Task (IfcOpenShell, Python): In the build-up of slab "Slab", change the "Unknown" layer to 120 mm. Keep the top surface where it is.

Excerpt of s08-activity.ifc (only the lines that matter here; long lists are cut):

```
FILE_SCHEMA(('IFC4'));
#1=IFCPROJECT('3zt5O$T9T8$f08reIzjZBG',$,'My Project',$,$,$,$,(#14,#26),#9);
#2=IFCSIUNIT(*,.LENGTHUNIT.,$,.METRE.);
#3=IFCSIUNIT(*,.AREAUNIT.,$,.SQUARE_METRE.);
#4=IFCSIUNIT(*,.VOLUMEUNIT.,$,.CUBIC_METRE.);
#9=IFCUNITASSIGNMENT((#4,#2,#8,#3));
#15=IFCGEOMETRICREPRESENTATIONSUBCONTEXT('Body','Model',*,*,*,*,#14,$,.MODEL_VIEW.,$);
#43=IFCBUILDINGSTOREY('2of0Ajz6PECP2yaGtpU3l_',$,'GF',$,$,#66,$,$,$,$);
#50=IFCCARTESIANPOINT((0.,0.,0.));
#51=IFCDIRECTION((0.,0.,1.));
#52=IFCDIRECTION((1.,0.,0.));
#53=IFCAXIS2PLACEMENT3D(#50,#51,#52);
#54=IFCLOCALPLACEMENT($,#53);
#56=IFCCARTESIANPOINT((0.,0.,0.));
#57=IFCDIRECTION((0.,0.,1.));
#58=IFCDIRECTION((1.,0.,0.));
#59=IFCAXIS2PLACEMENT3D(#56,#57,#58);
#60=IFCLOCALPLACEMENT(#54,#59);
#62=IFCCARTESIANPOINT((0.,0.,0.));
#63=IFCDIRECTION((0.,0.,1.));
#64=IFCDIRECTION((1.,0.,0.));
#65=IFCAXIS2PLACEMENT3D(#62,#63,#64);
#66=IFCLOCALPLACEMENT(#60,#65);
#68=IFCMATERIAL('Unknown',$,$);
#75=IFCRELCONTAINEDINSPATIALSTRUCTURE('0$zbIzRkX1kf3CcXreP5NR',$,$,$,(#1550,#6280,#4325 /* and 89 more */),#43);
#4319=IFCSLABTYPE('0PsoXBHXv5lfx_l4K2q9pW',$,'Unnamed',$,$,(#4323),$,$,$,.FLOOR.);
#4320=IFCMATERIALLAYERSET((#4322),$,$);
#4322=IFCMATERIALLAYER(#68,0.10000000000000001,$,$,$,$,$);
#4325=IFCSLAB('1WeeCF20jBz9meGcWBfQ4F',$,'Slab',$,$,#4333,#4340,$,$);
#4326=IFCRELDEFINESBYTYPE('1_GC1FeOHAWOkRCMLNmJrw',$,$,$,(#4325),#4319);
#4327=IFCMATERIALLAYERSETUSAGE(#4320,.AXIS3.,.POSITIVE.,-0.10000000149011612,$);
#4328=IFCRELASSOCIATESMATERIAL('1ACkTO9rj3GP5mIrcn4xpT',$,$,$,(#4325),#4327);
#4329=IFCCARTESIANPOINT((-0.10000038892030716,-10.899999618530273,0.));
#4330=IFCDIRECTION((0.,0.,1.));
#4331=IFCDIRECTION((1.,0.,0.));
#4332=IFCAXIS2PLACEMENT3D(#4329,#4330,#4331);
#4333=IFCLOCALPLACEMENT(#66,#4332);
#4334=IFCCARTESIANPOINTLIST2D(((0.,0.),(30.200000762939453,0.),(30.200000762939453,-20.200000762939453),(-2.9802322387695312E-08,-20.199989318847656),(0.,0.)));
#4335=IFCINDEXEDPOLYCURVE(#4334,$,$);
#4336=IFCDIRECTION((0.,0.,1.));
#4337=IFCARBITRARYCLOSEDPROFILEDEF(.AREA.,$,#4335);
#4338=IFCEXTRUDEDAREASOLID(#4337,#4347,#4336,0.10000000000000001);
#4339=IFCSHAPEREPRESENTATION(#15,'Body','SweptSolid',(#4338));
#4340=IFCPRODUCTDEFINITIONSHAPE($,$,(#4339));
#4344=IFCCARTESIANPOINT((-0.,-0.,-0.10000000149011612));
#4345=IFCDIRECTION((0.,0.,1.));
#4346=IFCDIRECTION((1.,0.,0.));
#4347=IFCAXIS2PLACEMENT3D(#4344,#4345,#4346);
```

```python
import ifcopenshell
import ifcopenshell.util.element
import ifcopenshell.util.representation
import ifcopenshell.util.unit

model = ifcopenshell.open("s08-activity.ifc")
unit_scale = ifcopenshell.util.unit.calculate_unit_scale(model)

layer_set = model.by_id(4320)
layer = next(l for l in layer_set.MaterialLayers if l.Material and l.Material.Name == "Unknown")
change = 0.12 / unit_scale - layer.LayerThickness
layer.LayerThickness += change

# Geometry does not follow the layer set by itself.
slabs = [e for e in ifcopenshell.util.element.get_elements_by_material(model, layer_set) if e.is_a("IfcSlab")]
for slab in sorted(slabs, key=lambda e: e.id()):
    body = ifcopenshell.util.representation.get_representation(slab, "Model", "Body")
    solid = body.Items[0]
    old_depth = solid.Depth
    solid.Depth += change
    # Extruded upwards: lower the start of the extrusion so the top stays.
    x, y, z = solid.Position.Location.Coordinates
    solid.Position.Location = model.createIfcCartesianPoint((x, y, z - change))
    print(slab.id(), f"{old_depth:g} -> {solid.Depth:g}")

# The layers are counted up from the underside, which has moved.
for usage in {ifcopenshell.util.element.get_material(slab) for slab in slabs}:
    usage.OffsetFromReferenceLine -= change

model.write("s08-activity_edited.ifc")
```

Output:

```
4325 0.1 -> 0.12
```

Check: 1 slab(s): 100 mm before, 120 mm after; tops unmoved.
